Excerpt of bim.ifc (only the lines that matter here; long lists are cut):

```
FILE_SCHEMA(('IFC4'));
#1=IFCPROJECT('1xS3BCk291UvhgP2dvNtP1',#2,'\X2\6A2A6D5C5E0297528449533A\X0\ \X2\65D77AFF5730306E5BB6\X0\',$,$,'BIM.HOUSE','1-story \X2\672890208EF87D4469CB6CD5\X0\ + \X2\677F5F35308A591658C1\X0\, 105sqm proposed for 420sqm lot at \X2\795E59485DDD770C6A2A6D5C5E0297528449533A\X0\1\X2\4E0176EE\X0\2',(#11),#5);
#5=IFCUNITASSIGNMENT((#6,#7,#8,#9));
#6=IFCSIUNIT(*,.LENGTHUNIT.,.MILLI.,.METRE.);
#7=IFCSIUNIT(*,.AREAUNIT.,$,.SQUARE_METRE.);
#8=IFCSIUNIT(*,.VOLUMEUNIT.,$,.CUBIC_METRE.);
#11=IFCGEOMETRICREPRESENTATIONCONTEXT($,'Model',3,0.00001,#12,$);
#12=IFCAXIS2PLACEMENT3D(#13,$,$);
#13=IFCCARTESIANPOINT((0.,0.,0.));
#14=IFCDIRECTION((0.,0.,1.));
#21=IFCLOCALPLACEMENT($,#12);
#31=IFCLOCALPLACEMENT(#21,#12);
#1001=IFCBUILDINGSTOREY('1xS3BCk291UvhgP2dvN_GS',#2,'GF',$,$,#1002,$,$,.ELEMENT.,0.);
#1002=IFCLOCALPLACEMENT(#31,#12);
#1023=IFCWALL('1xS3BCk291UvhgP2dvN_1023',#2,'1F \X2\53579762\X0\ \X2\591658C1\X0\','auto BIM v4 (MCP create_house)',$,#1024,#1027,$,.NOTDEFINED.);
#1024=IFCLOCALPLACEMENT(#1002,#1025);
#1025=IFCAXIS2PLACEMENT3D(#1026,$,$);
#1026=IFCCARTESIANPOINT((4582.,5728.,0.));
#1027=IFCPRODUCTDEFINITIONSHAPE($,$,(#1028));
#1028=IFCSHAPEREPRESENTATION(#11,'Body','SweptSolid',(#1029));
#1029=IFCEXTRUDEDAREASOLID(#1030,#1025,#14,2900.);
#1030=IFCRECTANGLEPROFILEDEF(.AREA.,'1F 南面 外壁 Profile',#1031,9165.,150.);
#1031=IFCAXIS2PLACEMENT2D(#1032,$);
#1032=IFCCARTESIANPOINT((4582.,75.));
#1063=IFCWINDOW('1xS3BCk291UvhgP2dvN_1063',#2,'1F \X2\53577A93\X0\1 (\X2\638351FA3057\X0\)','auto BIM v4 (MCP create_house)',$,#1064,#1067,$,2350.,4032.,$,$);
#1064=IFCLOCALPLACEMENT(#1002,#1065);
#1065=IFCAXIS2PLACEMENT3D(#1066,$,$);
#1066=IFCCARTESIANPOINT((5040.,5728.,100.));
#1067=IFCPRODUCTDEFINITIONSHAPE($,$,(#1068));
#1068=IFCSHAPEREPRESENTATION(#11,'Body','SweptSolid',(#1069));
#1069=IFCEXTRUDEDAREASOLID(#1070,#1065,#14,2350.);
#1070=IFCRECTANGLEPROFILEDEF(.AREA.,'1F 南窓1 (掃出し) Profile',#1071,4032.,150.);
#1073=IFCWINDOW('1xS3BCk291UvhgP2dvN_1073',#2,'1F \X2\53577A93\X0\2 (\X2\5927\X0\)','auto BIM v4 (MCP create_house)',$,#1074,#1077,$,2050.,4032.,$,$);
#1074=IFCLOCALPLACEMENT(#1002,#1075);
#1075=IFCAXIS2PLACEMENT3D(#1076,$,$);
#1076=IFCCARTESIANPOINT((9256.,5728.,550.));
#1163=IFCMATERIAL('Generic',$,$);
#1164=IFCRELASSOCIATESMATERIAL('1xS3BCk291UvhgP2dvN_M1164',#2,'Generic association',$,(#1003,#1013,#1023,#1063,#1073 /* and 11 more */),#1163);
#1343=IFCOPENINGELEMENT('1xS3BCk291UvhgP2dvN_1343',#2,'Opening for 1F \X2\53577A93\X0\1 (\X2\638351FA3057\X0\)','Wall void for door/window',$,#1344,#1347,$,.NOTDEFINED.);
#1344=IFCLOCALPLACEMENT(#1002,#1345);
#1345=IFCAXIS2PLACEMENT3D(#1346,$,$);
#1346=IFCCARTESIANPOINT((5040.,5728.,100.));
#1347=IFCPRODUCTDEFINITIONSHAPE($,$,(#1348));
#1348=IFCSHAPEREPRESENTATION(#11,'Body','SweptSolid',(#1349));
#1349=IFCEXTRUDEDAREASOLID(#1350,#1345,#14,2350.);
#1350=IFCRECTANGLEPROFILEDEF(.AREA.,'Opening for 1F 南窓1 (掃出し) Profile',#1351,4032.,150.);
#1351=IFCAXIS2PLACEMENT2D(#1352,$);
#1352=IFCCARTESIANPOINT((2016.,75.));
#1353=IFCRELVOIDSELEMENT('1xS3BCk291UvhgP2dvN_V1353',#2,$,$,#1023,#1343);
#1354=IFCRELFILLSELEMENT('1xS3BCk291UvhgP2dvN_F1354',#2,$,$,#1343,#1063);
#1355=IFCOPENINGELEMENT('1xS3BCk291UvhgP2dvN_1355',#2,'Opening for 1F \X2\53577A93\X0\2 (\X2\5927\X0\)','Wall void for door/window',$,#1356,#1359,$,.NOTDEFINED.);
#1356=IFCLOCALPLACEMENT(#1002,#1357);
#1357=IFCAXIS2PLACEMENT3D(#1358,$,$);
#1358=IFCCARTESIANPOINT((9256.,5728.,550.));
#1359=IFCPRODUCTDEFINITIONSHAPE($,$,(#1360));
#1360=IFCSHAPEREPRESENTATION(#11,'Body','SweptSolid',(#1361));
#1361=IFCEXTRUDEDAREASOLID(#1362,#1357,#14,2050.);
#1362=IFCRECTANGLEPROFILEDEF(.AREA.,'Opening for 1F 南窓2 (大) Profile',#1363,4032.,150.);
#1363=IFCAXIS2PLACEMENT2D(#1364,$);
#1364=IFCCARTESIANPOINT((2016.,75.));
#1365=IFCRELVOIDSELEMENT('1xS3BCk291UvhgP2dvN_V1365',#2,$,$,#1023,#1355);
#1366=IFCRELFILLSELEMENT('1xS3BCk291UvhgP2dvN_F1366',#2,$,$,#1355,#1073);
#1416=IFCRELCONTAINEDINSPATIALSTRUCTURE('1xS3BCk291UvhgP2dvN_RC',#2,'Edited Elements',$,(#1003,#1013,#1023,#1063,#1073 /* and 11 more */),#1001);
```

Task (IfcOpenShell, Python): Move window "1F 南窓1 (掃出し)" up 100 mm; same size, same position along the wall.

```python
import numpy as np
import ifcopenshell
import ifcopenshell.api.geometry
import ifcopenshell.util.placement
import ifcopenshell.util.unit

model = ifcopenshell.open("bim.ifc")
unit_scale = ifcopenshell.util.unit.calculate_unit_scale(model)

window = model.by_id(1063)
opening = window.FillsVoids[0].RelatingOpeningElement
dz = 0.1 / unit_scale

shift = np.array([0.0, 0.0, dz])
# The window is not placed relative to its opening, so move both.
for product in (opening, window):
    matrix = ifcopenshell.util.placement.get_local_placement(product.ObjectPlacement)
    matrix[:3, 3] += shift
    ifcopenshell.api.geometry.edit_object_placement(model, product=product, matrix=matrix, is_si=False)

print(f"moved by {dz * unit_scale:+.3f} m")

model.write("bim_edited.ifc")
```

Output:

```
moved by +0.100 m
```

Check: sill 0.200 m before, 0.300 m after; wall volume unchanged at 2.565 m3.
